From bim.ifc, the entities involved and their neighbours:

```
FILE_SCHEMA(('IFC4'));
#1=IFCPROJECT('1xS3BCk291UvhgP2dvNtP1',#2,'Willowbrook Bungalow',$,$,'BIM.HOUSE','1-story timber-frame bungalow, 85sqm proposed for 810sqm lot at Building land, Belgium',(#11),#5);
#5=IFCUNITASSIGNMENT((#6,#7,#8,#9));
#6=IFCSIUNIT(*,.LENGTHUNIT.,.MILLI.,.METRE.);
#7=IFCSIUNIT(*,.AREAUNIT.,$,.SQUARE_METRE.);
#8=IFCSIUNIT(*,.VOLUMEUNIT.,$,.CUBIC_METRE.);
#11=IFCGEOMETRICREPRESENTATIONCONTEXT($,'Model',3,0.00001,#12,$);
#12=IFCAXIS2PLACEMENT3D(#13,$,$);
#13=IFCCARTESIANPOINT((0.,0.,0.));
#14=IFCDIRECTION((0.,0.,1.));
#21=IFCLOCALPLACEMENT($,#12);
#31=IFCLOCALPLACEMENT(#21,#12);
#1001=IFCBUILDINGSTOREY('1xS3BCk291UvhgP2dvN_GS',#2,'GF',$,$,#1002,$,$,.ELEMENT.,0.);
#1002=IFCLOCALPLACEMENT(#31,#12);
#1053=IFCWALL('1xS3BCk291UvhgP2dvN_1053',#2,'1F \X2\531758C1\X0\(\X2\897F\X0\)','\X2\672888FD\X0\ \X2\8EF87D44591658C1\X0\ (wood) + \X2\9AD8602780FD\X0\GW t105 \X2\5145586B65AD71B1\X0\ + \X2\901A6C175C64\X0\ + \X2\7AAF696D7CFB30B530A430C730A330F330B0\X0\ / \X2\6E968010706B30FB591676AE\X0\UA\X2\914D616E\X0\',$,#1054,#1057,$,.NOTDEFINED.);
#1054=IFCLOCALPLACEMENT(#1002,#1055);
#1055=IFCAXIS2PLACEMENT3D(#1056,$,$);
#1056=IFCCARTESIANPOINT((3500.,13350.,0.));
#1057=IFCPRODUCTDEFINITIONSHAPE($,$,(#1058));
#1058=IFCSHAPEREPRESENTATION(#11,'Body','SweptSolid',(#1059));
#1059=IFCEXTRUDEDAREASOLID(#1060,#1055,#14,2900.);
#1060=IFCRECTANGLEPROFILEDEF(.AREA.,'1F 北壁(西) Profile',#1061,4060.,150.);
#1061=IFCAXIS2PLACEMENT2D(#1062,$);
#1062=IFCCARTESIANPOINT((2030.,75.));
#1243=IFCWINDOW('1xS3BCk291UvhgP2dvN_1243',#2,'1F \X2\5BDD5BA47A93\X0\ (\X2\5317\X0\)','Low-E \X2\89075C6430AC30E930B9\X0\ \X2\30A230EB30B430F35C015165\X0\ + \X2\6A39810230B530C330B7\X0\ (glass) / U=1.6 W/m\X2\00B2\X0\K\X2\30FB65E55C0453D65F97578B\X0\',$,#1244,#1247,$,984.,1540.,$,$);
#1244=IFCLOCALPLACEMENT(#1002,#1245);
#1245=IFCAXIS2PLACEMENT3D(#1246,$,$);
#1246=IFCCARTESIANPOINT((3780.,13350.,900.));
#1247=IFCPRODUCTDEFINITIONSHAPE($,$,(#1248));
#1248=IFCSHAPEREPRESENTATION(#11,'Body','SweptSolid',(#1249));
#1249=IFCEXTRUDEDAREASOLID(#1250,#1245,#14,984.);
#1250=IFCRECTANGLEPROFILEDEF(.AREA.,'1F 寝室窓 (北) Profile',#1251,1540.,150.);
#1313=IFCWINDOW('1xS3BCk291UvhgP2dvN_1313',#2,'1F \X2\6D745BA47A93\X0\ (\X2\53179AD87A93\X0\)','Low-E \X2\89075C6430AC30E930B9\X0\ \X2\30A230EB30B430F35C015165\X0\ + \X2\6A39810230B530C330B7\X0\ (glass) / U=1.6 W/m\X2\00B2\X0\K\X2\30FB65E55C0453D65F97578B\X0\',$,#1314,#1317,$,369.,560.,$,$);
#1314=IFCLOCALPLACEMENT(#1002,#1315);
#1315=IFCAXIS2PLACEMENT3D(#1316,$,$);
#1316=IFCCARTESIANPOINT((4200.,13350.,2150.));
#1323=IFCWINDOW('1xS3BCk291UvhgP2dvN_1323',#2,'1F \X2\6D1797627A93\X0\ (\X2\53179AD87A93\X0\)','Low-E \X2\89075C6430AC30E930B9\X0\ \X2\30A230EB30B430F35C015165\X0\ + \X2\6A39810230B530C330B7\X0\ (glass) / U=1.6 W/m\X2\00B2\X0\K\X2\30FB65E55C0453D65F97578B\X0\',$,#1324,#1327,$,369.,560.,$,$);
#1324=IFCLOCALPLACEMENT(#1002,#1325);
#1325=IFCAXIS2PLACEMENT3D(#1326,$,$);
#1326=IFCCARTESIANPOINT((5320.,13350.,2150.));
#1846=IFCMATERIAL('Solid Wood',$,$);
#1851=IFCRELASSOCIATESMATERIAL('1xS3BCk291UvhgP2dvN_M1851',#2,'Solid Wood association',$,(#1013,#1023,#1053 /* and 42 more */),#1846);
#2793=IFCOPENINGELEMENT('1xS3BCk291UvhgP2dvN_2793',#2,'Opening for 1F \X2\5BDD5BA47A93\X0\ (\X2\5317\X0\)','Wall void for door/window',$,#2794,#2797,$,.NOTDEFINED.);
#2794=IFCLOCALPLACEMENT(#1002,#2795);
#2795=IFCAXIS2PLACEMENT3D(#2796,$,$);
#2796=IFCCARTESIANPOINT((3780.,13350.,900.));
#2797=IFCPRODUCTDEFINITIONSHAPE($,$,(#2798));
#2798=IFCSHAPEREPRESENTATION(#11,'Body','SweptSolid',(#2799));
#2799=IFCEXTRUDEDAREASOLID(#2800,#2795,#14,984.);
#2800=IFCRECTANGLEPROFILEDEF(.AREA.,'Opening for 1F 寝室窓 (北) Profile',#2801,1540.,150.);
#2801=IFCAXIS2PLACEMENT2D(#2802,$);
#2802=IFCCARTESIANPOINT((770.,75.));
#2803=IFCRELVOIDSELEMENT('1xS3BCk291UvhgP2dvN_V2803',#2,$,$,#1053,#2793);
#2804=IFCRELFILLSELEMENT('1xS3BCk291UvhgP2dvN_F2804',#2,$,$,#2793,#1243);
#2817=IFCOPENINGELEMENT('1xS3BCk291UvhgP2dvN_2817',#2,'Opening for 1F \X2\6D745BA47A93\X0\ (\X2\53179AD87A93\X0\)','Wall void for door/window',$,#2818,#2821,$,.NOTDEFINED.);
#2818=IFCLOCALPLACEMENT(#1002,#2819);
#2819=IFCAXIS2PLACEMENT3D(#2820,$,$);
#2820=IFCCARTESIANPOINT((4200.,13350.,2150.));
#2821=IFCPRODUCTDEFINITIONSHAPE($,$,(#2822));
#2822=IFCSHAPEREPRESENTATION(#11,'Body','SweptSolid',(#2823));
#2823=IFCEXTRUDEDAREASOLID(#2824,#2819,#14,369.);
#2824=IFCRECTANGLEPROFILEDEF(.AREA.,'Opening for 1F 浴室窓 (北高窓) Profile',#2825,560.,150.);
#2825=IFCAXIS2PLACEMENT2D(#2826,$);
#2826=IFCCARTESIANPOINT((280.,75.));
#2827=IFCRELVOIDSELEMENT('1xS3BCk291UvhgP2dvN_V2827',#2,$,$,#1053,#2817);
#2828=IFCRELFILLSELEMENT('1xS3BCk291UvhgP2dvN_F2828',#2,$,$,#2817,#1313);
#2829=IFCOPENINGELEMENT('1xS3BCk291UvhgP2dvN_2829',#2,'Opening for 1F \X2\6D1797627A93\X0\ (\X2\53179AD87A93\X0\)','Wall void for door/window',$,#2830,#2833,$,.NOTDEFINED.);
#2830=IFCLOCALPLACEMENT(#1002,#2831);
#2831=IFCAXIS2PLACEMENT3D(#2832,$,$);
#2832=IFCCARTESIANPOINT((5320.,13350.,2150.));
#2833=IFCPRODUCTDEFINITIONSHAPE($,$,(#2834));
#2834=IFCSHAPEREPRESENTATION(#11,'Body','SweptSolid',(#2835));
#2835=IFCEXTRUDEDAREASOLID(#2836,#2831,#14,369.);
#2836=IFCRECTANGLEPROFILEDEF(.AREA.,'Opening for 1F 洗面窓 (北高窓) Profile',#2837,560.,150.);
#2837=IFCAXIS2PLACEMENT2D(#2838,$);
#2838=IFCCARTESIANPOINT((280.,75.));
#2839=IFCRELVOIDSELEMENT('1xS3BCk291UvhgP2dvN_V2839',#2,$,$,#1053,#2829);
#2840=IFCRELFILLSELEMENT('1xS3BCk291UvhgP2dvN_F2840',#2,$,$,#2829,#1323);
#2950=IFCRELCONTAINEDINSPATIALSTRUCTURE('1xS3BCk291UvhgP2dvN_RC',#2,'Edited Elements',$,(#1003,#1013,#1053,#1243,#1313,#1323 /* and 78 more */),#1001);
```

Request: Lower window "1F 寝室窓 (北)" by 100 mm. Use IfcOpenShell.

```python
import numpy as np
import ifcopenshell
import ifcopenshell.api.geometry
import ifcopenshell.util.placement
import ifcopenshell.util.unit

model = ifcopenshell.open("bim.ifc")
unit_scale = ifcopenshell.util.unit.calculate_unit_scale(model)

window = model.by_guid("1xS3BCk291UvhgP2dvN_1243")
opening = window.FillsVoids[0].RelatingOpeningElement
dz = -0.1 / unit_scale

shift = np.array([0.0, 0.0, dz])
# The window is not placed relative to its opening, so move both.
for product in (opening, window):
    matrix = ifcopenshell.util.placement.get_local_placement(product.ObjectPlacement)
    matrix[:3, 3] += shift
    ifcopenshell.api.geometry.edit_object_placement(model, product=product, matrix=matrix, is_si=False)

print(f"moved by {dz * unit_scale:+.3f} m")

model.write("bim-out.ifc")
```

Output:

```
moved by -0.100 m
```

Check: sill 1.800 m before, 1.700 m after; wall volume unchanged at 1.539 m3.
